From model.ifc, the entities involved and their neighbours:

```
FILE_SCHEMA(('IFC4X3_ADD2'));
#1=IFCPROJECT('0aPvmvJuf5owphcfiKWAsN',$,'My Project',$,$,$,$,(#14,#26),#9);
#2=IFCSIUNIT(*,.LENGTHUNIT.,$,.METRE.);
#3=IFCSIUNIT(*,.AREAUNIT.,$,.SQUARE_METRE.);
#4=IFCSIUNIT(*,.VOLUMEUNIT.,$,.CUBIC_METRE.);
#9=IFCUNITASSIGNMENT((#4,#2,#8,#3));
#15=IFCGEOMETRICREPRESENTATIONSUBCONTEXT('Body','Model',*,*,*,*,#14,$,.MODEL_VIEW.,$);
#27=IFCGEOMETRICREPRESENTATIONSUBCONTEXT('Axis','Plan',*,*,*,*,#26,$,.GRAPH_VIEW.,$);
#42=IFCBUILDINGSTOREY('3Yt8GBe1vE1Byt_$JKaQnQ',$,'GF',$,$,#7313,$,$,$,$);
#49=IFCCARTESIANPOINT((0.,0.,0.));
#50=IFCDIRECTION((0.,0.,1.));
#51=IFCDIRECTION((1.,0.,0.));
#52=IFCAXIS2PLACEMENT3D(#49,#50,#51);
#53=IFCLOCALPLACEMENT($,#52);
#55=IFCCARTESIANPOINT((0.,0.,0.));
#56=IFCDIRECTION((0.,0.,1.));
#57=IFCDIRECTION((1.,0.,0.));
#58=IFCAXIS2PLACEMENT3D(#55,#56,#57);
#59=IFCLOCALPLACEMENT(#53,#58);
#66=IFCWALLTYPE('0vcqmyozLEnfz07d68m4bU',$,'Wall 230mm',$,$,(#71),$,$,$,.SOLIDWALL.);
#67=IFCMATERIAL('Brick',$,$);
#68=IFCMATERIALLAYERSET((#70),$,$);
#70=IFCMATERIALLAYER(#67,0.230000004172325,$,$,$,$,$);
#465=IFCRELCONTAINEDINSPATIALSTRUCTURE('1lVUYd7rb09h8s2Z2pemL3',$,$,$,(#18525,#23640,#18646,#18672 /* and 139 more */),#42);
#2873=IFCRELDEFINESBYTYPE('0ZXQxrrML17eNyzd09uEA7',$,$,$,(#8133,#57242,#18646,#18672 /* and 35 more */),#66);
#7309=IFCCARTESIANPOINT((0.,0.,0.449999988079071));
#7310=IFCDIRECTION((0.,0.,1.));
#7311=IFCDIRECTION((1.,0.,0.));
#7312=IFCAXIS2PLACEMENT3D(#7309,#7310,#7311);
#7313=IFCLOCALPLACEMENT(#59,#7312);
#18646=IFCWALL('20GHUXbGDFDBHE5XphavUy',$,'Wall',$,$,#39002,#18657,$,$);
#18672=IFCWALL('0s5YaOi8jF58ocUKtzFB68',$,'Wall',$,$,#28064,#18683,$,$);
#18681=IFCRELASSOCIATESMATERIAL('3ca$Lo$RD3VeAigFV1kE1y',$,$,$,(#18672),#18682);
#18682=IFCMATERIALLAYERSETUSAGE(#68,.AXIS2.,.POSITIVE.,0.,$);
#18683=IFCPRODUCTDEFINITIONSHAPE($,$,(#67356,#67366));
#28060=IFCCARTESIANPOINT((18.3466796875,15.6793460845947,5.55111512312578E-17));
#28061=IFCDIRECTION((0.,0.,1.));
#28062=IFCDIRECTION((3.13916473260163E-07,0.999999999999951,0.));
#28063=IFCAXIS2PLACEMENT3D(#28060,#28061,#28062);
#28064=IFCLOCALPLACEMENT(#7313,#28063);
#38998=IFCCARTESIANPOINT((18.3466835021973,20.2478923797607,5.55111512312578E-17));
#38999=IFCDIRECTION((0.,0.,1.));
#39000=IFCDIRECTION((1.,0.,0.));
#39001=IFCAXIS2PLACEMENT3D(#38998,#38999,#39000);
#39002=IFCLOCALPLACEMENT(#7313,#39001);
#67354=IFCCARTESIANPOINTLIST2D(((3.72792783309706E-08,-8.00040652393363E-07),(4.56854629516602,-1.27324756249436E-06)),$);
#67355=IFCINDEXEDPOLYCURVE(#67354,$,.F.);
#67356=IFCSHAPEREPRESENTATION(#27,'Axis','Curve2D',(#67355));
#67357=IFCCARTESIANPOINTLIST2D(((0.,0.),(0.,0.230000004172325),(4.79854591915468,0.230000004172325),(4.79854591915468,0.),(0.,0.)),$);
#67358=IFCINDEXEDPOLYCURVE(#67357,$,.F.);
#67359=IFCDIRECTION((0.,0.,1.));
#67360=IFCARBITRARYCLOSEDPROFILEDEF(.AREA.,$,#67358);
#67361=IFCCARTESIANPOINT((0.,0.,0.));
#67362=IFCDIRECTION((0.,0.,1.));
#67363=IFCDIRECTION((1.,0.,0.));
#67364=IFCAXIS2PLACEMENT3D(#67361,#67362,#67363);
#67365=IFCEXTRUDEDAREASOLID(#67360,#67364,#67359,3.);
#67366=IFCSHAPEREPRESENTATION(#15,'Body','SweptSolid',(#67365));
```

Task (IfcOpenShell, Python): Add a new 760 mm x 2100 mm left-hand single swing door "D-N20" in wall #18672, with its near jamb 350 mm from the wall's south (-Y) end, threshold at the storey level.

```python
import numpy as np
import ifcopenshell
import ifcopenshell.api.feature
import ifcopenshell.api.geometry
import ifcopenshell.api.root
import ifcopenshell.api.spatial
import ifcopenshell.geom
import ifcopenshell.util.element
import ifcopenshell.util.placement
import ifcopenshell.util.representation
import ifcopenshell.util.shape
import ifcopenshell.util.unit

model = ifcopenshell.open("model.ifc")
unit_scale = ifcopenshell.util.unit.calculate_unit_scale(model)
settings = ifcopenshell.geom.settings()


def volume(element):
    """Net volume in cubic metres, openings subtracted."""
    shape = ifcopenshell.geom.create_shape(settings, element)
    return ifcopenshell.util.shape.get_volume(shape.geometry)


wall = model.by_id(18672)
storey = ifcopenshell.util.element.get_container(wall, ifc_class="IfcBuildingStorey")
context = ifcopenshell.util.representation.get_context(model, "Model", "Body", "MODEL_VIEW")
before = volume(wall)

width, height, from_end, sill = 0.76, 2.1, 0.35, 0.0  # metres

# The wall runs along its own X axis, and the end named is its -X end.
wall_shape = ifcopenshell.geom.create_shape(settings, wall)
x, y, z = ifcopenshell.util.shape.get_vertices(wall_shape.geometry).T
start = x.min() + from_end
face, thickness = float(y.min()), float(y.max() - y.min())
wall_matrix = ifcopenshell.util.placement.get_local_placement(wall.ObjectPlacement)
level = ifcopenshell.util.placement.get_local_placement(storey.ObjectPlacement)[2, 3]


def in_wall(x, y):
    """Placement at x, y metres in the wall's axes, at sill height."""
    matrix = wall_matrix.copy()
    matrix[:, 3] = wall_matrix @ np.array([x / unit_scale, y / unit_scale, 0.0, 1.0])
    matrix[2, 3] = level + sill / unit_scale
    return matrix


# Opening: a box that overshoots both wall faces by 50 mm.
opening = ifcopenshell.api.root.create_entity(model, ifc_class="IfcOpeningElement", predefined_type="OPENING")
box = ifcopenshell.api.geometry.add_wall_representation(
    model, context=context, length=width, height=height, thickness=thickness + 0.1
)
ifcopenshell.api.geometry.assign_representation(model, product=opening, representation=box)
ifcopenshell.api.geometry.edit_object_placement(model, product=opening, matrix=in_wall(start, face - 0.05), is_si=False)
ifcopenshell.api.feature.add_feature(model, feature=opening, element=wall)

door = ifcopenshell.api.root.create_entity(model, ifc_class="IfcDoor", name="D-N20", predefined_type="DOOR")
door.OverallWidth, door.OverallHeight = width / unit_scale, height / unit_scale
door.OperationType = "SINGLE_SWING_LEFT"
body = ifcopenshell.api.geometry.add_door_representation(
    model,
    context=context,
    overall_width=door.OverallWidth,
    overall_height=door.OverallHeight,
    operation_type="SINGLE_SWING_LEFT",
    lining_properties={"LiningDepth": thickness / unit_scale, "ThresholdDepth": thickness / unit_scale},
)
ifcopenshell.api.geometry.assign_representation(model, product=door, representation=body)
ifcopenshell.api.spatial.assign_container(model, products=[door], relating_structure=storey)
ifcopenshell.api.feature.add_filling(model, opening=opening, element=door)

# The lining spans the wall, so the door starts at the wall face.
ifcopenshell.api.geometry.edit_object_placement(model, product=door, matrix=in_wall(start, face), is_si=False)

after = volume(wall)

print(f"wall volume {before:.3f} -> {after:.3f} m3")

model.write("model_edited.ifc")
```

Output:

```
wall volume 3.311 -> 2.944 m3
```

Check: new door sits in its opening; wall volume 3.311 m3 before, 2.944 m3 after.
